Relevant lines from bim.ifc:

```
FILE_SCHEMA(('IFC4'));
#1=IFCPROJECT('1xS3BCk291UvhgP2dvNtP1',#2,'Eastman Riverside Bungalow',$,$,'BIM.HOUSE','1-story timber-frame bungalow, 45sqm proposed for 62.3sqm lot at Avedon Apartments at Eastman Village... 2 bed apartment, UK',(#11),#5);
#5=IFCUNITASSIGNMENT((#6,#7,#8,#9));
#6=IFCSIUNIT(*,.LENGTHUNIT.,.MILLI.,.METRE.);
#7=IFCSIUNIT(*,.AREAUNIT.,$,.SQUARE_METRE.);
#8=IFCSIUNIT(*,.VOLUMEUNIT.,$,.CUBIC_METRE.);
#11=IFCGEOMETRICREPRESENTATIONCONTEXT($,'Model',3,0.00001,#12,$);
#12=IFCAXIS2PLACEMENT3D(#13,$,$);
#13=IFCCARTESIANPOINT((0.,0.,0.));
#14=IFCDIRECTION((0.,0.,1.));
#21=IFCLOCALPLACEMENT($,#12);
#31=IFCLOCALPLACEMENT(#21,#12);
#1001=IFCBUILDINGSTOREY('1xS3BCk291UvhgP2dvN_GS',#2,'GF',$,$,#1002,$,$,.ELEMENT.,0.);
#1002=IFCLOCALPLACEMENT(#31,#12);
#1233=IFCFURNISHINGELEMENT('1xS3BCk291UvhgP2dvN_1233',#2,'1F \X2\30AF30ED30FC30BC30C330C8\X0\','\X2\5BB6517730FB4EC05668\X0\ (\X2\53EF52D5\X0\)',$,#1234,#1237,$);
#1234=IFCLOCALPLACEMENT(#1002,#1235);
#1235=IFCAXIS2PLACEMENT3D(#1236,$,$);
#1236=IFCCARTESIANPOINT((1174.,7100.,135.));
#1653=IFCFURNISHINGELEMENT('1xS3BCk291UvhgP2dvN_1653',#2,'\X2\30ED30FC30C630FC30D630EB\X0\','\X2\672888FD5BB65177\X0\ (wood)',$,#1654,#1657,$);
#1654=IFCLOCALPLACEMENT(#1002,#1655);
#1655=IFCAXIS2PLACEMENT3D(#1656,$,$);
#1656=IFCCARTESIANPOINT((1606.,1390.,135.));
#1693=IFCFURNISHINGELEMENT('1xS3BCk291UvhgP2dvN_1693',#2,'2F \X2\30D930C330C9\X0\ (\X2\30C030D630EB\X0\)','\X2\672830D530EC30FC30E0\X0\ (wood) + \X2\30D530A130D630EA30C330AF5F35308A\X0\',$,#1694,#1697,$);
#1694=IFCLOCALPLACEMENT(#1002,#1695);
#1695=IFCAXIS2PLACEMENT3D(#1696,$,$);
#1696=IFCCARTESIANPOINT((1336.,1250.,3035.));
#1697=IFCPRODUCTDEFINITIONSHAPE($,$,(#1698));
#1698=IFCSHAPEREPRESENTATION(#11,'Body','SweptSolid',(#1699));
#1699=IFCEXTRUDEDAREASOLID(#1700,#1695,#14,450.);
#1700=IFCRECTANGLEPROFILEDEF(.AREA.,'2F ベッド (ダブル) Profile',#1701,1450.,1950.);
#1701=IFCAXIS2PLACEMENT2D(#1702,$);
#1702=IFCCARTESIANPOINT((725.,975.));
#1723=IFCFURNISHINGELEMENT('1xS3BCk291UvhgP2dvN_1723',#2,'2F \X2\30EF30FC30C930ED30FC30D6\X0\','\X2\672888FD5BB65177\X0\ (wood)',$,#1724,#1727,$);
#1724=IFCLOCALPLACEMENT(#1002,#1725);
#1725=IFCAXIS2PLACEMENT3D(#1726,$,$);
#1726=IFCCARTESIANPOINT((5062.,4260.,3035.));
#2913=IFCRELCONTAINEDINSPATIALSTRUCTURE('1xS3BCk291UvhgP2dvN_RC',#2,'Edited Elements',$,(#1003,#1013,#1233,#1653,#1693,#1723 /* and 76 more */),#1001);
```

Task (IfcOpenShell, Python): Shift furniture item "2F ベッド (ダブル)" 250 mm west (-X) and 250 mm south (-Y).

```python
import ifcopenshell
import ifcopenshell.api.geometry
import ifcopenshell.util.placement

model = ifcopenshell.open("bim.ifc")

item = model.by_guid("1xS3BCk291UvhgP2dvN_1693")
matrix = ifcopenshell.util.placement.get_local_placement(item.ObjectPlacement)
matrix[0, 3] -= 250.0
matrix[1, 3] -= 250.0
ifcopenshell.api.geometry.edit_object_placement(model, product=item, matrix=matrix, is_si=False)

print(ifcopenshell.util.placement.get_local_placement(item.ObjectPlacement).round(3) + 0.0)

model.write("bim-out.ifc")
```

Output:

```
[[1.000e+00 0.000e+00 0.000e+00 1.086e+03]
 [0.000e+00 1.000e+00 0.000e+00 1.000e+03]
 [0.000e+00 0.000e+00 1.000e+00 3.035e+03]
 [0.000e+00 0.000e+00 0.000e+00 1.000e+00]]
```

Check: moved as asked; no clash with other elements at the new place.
